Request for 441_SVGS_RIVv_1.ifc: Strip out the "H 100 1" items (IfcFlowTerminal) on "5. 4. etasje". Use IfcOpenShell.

First a look at what the model holds.

```python
import ifcopenshell
import ifcopenshell.util.element

model = ifcopenshell.open("441_SVGS_RIVv_1.ifc")
print(model.schema)
storey = next(s for s in model.by_type("IfcBuildingStorey") if s.Name == "5. 4. etasje")
terminals = [e for e in ifcopenshell.util.element.get_decomposition(storey) if e.is_a("IfcFlowTerminal")]
seen = {}
for e in terminals:
    element_type = ifcopenshell.util.element.get_type(e)
    name = element_type.Name if element_type not in (None, e) else None
    seen[name] = seen.get(name, 0) + 1
for name, count in sorted(seen.items(), key=str):
    print(count, "x", name)
```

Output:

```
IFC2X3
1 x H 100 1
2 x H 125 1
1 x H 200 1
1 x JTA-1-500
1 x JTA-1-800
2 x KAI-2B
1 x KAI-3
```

```python
import ifcopenshell
import ifcopenshell.api.root
import ifcopenshell.util.element

model = ifcopenshell.open("441_SVGS_RIVv_1.ifc")

storey = next(s for s in model.by_type("IfcBuildingStorey") if s.Name == "5. 4. etasje")
terminals = [e for e in ifcopenshell.util.element.get_decomposition(storey) if e.is_a("IfcFlowTerminal")]
targets = [e for e in terminals if (t := ifcopenshell.util.element.get_type(e)) not in (None, e) and t.Name == "H 100 1"]

for e in targets:
    ifcopenshell.api.root.remove_product(model, product=e)
print(len(targets), "removed")

model.write("441_SVGS_RIVv_1_rev.ifc")
```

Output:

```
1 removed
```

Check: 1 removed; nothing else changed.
